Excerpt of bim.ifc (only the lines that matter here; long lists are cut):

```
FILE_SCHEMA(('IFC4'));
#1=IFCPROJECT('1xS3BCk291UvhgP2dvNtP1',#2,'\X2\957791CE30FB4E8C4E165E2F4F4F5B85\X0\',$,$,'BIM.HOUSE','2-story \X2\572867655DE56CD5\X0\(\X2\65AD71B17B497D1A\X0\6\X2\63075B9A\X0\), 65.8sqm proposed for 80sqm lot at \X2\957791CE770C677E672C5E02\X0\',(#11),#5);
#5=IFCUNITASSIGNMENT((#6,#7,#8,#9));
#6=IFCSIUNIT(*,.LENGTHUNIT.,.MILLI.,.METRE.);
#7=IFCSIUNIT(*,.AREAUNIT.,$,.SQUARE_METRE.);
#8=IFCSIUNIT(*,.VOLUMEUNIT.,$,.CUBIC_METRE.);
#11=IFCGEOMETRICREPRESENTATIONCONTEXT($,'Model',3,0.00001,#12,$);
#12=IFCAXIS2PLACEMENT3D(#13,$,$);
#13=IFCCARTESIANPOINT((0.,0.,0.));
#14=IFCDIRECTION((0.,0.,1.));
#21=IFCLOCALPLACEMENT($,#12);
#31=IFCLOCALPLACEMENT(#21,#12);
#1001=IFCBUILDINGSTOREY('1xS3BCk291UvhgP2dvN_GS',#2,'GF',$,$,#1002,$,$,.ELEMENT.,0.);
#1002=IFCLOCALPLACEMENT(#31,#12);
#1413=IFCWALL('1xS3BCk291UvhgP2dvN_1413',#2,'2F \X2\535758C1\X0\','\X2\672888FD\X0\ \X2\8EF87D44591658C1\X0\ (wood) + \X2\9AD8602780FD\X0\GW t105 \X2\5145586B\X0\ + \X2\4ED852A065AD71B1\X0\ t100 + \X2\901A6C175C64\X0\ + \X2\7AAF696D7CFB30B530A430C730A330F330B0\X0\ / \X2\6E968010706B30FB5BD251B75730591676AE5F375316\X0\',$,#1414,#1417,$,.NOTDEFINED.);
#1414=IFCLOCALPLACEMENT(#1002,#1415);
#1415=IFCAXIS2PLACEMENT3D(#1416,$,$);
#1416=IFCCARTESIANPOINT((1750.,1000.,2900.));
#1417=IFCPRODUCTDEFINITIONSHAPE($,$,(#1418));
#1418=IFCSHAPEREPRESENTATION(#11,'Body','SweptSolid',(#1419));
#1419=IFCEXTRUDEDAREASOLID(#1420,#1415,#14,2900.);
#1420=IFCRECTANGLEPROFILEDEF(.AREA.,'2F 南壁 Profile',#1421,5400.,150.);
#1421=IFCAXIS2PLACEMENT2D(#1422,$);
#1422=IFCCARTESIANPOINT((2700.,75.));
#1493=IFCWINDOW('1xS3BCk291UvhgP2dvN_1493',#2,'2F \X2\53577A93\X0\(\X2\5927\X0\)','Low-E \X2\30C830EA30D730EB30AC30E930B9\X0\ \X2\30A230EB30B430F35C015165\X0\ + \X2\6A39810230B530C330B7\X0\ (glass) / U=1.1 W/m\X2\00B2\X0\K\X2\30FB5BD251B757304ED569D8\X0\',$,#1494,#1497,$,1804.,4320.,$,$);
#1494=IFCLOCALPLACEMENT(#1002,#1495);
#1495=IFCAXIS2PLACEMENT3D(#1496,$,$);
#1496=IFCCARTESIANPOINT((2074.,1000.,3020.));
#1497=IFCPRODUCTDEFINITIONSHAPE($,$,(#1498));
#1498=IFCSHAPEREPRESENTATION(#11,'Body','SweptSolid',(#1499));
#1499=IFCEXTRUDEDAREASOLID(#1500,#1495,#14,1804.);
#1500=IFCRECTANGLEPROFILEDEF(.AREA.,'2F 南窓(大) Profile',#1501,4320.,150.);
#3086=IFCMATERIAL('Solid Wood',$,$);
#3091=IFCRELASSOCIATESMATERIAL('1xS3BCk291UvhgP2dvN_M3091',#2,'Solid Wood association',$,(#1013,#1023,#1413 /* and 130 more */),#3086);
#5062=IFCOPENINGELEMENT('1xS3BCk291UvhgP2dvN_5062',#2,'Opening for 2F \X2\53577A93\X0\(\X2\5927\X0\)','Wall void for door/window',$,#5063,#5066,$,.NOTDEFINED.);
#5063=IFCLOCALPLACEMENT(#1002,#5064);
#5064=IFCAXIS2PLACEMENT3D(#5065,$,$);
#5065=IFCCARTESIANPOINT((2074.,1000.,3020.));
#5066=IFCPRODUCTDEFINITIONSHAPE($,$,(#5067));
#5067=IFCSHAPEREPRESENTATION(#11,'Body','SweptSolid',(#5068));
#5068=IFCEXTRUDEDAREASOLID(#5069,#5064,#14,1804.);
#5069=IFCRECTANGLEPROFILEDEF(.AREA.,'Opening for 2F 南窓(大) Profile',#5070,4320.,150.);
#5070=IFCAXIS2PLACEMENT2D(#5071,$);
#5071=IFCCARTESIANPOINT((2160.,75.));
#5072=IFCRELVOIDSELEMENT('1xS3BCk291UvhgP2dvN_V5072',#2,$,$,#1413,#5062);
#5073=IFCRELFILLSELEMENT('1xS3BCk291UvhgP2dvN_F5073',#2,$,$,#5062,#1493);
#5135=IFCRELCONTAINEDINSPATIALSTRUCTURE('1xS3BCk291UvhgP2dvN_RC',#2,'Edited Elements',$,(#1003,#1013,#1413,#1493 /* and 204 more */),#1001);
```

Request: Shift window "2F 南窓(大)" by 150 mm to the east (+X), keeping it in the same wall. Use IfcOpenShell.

```python
import ifcopenshell
import ifcopenshell.api.geometry
import ifcopenshell.util.placement
import ifcopenshell.util.unit

model = ifcopenshell.open("bim.ifc")
unit_scale = ifcopenshell.util.unit.calculate_unit_scale(model)

window = model.by_id(1493)
opening = window.FillsVoids[0].RelatingOpeningElement
wall = opening.VoidsElements[0].RelatingBuildingElement

wall_matrix = ifcopenshell.util.placement.get_local_placement(wall.ObjectPlacement)
shift = wall_matrix[:3, 0] * 0.15 / unit_scale
before = ifcopenshell.util.placement.get_local_placement(window.ObjectPlacement)[:3, 3].copy()

# The window is not placed relative to its opening, so move both.
for product in (opening, window):
    matrix = ifcopenshell.util.placement.get_local_placement(product.ObjectPlacement)
    matrix[:3, 3] += shift
    ifcopenshell.api.geometry.edit_object_placement(model, product=product, matrix=matrix, is_si=False)

after = ifcopenshell.util.placement.get_local_placement(window.ObjectPlacement)[:3, 3]
print("window moved by", (after - before).round(3) + 0.0)

model.write("bim-out.ifc")
```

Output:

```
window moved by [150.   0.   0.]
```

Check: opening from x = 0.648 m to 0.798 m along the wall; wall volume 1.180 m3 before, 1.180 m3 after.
